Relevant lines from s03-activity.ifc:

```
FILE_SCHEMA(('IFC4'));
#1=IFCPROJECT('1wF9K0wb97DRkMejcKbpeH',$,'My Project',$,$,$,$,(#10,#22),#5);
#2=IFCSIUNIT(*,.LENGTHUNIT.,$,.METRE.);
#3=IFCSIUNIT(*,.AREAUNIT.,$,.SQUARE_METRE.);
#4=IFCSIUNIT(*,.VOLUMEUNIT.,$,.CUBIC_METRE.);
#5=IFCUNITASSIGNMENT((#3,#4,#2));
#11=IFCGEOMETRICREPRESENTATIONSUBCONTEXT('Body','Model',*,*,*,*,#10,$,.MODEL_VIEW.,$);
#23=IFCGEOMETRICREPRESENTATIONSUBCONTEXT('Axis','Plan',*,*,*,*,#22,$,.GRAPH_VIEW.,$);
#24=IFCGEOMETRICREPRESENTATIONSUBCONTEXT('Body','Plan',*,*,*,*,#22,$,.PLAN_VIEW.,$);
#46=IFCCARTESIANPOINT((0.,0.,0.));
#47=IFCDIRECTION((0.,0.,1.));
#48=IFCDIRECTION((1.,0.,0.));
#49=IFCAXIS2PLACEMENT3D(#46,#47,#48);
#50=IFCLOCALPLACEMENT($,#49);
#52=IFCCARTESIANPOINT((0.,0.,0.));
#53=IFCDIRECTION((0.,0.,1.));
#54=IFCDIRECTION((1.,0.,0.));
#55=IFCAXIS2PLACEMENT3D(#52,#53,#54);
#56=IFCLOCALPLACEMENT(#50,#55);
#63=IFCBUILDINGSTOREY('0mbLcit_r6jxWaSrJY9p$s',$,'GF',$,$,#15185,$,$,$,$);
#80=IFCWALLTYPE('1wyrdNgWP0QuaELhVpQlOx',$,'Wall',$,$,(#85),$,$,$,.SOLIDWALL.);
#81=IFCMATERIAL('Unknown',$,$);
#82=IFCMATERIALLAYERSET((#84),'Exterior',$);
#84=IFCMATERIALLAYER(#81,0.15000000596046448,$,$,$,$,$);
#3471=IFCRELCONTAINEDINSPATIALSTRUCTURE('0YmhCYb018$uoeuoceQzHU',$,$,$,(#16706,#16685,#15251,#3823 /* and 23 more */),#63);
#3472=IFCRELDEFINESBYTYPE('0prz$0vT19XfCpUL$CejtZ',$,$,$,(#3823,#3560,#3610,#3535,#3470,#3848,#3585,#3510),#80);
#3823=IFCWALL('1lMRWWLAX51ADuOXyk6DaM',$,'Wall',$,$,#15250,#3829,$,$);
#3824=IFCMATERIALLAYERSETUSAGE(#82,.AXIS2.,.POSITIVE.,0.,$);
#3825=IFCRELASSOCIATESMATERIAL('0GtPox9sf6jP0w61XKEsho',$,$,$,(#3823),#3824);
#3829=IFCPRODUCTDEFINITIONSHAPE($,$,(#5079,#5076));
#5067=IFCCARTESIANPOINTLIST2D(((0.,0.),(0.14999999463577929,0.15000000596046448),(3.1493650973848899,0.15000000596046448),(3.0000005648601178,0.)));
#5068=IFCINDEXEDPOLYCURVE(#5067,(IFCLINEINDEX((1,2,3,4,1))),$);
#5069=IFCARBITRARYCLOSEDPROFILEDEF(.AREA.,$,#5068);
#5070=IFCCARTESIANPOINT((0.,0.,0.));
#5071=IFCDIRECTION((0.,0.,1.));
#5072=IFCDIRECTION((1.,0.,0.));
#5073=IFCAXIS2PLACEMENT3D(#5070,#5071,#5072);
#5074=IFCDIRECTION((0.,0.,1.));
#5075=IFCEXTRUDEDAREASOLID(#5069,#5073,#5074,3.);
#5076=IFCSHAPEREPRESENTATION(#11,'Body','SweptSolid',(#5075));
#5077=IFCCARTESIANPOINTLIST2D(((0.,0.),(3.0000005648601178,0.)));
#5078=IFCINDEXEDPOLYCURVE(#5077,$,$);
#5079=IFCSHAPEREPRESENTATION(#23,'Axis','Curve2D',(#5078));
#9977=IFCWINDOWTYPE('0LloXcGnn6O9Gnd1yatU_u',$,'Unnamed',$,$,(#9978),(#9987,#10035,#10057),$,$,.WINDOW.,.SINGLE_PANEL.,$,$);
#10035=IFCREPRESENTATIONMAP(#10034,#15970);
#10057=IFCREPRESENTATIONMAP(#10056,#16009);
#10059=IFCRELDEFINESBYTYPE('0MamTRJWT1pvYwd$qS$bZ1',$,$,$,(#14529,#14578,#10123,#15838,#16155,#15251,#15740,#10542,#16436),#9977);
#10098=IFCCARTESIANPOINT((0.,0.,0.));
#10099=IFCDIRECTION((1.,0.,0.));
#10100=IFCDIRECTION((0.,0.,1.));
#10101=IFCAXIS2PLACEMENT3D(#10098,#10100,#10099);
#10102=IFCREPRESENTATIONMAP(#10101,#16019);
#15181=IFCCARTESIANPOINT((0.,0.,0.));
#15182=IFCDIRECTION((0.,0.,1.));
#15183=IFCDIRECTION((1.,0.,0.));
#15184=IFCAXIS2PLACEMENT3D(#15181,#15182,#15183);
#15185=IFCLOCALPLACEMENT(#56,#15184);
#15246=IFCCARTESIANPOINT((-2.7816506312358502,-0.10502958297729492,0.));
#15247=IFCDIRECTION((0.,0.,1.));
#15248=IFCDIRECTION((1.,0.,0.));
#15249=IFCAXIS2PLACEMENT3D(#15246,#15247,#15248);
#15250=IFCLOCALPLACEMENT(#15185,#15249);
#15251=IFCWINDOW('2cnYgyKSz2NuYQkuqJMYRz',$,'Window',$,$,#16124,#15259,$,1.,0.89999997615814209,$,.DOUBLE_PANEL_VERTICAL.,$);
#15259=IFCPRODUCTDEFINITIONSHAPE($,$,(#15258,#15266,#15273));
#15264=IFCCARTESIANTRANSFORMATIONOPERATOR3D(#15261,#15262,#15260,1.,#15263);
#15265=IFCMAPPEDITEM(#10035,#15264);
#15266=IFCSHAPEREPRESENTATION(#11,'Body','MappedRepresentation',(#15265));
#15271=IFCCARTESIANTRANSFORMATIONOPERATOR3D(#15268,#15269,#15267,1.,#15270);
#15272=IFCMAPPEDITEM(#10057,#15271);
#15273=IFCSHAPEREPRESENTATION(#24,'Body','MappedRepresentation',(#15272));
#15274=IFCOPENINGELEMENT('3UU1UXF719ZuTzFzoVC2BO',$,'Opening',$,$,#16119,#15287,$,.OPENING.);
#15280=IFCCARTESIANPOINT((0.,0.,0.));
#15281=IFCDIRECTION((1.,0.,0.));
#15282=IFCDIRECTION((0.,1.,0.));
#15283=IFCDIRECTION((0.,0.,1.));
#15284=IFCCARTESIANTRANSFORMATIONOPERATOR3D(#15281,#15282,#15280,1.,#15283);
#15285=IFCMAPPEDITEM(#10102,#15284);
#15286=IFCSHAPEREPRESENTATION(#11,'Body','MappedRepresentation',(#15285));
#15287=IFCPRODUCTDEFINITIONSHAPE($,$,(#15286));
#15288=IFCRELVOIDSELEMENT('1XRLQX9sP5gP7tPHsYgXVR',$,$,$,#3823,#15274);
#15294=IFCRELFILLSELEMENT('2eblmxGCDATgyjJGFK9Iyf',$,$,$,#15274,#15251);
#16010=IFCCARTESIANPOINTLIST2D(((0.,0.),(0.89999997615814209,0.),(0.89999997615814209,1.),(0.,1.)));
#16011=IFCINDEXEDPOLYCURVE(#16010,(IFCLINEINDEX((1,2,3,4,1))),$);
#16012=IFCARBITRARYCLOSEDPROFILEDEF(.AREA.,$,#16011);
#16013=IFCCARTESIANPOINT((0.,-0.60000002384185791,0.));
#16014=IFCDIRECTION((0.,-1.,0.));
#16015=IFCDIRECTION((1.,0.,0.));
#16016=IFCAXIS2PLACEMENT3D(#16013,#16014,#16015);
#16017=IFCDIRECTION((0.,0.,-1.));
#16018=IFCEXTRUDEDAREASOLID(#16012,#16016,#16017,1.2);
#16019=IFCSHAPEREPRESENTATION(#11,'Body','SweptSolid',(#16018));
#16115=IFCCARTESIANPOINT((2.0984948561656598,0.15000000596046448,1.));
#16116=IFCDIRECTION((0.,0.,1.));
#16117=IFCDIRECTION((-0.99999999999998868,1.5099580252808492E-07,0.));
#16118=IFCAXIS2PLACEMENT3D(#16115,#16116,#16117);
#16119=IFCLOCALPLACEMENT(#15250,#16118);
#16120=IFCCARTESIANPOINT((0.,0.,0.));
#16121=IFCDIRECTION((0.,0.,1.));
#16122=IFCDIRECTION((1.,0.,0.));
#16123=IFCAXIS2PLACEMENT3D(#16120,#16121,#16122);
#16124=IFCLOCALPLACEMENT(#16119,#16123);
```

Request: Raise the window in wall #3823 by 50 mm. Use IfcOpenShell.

```python
import numpy as np
import ifcopenshell
import ifcopenshell.api.geometry
import ifcopenshell.util.placement
import ifcopenshell.util.unit

model = ifcopenshell.open("s03-activity.ifc")
unit_scale = ifcopenshell.util.unit.calculate_unit_scale(model)

window = model.by_guid("2cnYgyKSz2NuYQkuqJMYRz")
opening = window.FillsVoids[0].RelatingOpeningElement
dz = 0.05

shift = np.array([0.0, 0.0, dz])
# The window is placed relative to its opening, so it follows when the opening moves.
matrix = ifcopenshell.util.placement.get_local_placement(opening.ObjectPlacement)
matrix[:3, 3] += shift
ifcopenshell.api.geometry.edit_object_placement(
    model, product=opening, matrix=matrix, is_si=False, should_transform_children=True
)

print(f"moved by {dz * unit_scale:+.3f} m")

model.write("s03-activity_edited.ifc")
```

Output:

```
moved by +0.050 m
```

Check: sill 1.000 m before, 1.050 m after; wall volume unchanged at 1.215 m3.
